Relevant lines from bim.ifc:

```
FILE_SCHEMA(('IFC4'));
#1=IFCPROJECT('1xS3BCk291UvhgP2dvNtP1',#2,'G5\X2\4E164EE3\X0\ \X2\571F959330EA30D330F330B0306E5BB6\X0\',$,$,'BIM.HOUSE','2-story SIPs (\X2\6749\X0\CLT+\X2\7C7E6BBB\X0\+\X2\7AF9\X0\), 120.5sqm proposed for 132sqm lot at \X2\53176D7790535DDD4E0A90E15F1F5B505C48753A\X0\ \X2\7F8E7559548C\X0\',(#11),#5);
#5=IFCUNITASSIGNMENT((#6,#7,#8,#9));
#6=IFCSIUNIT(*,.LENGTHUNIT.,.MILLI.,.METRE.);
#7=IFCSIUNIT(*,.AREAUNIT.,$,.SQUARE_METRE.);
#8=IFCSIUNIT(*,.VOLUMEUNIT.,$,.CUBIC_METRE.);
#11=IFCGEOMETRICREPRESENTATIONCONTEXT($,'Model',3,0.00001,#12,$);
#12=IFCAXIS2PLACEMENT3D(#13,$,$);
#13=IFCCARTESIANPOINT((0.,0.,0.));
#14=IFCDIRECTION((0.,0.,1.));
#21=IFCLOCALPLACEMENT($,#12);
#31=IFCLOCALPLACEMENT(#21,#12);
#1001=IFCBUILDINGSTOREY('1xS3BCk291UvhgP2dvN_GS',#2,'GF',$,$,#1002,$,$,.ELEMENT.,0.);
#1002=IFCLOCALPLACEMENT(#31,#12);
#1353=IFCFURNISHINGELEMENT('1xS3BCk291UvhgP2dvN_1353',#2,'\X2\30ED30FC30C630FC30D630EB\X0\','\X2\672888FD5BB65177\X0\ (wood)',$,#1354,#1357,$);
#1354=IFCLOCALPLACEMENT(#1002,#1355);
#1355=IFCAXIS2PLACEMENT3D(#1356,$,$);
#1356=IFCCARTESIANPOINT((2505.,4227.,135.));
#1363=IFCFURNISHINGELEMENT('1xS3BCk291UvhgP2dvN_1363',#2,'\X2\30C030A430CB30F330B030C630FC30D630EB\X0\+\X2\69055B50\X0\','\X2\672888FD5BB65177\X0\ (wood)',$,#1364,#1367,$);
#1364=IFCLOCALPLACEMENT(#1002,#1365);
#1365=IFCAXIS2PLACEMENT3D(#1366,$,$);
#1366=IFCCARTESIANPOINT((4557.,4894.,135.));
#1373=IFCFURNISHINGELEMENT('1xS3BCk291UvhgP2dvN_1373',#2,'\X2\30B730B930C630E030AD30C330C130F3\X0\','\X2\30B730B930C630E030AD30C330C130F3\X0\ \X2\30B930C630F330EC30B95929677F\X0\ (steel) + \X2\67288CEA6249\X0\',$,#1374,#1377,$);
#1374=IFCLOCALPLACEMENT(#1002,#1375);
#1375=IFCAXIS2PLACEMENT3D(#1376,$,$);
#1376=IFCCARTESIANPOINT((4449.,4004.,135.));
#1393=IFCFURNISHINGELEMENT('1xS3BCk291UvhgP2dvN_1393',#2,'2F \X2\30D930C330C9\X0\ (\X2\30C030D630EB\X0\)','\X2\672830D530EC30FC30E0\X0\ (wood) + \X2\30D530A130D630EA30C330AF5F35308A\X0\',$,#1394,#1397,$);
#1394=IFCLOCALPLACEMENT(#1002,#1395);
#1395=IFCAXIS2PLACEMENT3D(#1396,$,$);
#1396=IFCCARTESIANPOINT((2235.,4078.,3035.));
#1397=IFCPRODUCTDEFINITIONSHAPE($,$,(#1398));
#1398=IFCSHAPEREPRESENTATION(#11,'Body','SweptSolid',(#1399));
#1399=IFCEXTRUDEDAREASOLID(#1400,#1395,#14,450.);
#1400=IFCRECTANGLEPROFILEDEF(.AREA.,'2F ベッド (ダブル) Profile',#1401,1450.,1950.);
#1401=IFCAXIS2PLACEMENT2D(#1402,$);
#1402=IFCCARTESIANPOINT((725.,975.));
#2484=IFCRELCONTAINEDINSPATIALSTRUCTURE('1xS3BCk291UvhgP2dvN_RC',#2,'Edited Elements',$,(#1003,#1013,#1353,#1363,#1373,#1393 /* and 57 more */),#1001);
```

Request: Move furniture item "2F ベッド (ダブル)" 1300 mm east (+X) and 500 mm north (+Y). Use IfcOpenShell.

```python
import ifcopenshell
import ifcopenshell.api.geometry
import ifcopenshell.util.placement
import ifcopenshell.util.unit

model = ifcopenshell.open("bim.ifc")
unit_scale = ifcopenshell.util.unit.calculate_unit_scale(model)

item = model.by_guid("1xS3BCk291UvhgP2dvN_1393")
matrix = ifcopenshell.util.placement.get_local_placement(item.ObjectPlacement)
matrix[0, 3] += 1.3 / unit_scale
matrix[1, 3] += 0.5 / unit_scale
ifcopenshell.api.geometry.edit_object_placement(model, product=item, matrix=matrix, is_si=False)

print(ifcopenshell.util.placement.get_local_placement(item.ObjectPlacement).round(3) + 0.0)

model.write("bim_edited.ifc")
```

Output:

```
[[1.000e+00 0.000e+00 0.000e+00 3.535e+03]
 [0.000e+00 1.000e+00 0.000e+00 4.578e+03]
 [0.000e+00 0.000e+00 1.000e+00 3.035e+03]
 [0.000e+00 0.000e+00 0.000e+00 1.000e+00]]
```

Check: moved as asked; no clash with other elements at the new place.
